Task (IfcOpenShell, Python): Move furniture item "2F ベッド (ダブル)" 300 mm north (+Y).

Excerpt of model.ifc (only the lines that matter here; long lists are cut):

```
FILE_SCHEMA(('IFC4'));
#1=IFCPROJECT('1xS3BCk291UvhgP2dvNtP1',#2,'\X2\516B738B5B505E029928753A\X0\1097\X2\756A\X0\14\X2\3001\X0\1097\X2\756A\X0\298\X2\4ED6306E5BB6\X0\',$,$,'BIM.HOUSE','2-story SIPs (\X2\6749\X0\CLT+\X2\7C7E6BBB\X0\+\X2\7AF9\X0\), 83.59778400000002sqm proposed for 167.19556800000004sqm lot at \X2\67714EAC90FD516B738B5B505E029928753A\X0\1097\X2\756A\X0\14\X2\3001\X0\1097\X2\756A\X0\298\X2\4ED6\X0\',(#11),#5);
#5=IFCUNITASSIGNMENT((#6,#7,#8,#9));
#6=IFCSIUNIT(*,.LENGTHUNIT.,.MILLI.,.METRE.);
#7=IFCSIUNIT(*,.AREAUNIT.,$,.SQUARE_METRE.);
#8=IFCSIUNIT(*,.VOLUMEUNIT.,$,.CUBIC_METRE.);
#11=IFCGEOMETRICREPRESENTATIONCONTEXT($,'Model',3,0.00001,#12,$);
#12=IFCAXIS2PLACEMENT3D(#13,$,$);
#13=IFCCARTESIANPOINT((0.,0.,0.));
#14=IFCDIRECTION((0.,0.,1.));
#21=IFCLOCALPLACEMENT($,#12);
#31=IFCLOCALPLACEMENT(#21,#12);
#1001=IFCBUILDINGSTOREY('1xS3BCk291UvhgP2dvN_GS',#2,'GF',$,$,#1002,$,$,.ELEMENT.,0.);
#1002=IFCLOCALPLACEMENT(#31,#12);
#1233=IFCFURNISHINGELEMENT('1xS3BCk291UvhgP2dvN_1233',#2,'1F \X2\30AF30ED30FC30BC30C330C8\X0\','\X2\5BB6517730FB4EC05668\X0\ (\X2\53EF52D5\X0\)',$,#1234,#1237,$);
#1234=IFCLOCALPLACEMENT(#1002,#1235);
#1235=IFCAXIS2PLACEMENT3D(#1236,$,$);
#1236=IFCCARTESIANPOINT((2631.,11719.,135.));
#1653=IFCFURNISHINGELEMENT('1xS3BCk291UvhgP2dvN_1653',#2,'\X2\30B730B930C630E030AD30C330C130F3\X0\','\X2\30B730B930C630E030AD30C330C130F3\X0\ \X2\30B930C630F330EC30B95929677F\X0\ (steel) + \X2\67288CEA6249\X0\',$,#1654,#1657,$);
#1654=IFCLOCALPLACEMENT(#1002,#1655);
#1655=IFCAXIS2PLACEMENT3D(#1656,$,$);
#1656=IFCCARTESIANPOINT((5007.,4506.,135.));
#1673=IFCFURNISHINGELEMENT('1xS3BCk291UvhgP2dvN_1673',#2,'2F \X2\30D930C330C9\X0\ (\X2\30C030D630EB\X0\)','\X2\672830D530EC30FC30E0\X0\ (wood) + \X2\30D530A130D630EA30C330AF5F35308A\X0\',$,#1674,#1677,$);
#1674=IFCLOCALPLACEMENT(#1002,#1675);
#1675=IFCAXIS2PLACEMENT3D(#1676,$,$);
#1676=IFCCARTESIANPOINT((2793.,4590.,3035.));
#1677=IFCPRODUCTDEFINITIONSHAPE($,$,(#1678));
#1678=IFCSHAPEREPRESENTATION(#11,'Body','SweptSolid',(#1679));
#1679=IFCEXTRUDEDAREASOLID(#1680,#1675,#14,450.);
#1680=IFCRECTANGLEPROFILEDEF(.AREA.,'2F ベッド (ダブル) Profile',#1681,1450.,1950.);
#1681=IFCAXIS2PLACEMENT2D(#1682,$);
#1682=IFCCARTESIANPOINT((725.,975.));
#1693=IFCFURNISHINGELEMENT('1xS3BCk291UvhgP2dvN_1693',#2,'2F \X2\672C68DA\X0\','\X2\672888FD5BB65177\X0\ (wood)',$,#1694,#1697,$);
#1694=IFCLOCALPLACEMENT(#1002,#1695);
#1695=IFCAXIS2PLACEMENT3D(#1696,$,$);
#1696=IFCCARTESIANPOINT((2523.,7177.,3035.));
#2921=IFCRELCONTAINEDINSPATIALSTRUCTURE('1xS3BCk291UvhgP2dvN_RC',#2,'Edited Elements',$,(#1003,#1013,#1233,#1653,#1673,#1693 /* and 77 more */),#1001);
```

```python
import ifcopenshell
import ifcopenshell.api.geometry
import ifcopenshell.util.placement
import ifcopenshell.util.unit

model = ifcopenshell.open("model.ifc")
unit_scale = ifcopenshell.util.unit.calculate_unit_scale(model)

item = model.by_guid("1xS3BCk291UvhgP2dvN_1673")
matrix = ifcopenshell.util.placement.get_local_placement(item.ObjectPlacement)
matrix[1, 3] += 0.3 / unit_scale
ifcopenshell.api.geometry.edit_object_placement(model, product=item, matrix=matrix, is_si=False)

print(ifcopenshell.util.placement.get_local_placement(item.ObjectPlacement).round(3) + 0.0)

model.write("model_rev.ifc")
```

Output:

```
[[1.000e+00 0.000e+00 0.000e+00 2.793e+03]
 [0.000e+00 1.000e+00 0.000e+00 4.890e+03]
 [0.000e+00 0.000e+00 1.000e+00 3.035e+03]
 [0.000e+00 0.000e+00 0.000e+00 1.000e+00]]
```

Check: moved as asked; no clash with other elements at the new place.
